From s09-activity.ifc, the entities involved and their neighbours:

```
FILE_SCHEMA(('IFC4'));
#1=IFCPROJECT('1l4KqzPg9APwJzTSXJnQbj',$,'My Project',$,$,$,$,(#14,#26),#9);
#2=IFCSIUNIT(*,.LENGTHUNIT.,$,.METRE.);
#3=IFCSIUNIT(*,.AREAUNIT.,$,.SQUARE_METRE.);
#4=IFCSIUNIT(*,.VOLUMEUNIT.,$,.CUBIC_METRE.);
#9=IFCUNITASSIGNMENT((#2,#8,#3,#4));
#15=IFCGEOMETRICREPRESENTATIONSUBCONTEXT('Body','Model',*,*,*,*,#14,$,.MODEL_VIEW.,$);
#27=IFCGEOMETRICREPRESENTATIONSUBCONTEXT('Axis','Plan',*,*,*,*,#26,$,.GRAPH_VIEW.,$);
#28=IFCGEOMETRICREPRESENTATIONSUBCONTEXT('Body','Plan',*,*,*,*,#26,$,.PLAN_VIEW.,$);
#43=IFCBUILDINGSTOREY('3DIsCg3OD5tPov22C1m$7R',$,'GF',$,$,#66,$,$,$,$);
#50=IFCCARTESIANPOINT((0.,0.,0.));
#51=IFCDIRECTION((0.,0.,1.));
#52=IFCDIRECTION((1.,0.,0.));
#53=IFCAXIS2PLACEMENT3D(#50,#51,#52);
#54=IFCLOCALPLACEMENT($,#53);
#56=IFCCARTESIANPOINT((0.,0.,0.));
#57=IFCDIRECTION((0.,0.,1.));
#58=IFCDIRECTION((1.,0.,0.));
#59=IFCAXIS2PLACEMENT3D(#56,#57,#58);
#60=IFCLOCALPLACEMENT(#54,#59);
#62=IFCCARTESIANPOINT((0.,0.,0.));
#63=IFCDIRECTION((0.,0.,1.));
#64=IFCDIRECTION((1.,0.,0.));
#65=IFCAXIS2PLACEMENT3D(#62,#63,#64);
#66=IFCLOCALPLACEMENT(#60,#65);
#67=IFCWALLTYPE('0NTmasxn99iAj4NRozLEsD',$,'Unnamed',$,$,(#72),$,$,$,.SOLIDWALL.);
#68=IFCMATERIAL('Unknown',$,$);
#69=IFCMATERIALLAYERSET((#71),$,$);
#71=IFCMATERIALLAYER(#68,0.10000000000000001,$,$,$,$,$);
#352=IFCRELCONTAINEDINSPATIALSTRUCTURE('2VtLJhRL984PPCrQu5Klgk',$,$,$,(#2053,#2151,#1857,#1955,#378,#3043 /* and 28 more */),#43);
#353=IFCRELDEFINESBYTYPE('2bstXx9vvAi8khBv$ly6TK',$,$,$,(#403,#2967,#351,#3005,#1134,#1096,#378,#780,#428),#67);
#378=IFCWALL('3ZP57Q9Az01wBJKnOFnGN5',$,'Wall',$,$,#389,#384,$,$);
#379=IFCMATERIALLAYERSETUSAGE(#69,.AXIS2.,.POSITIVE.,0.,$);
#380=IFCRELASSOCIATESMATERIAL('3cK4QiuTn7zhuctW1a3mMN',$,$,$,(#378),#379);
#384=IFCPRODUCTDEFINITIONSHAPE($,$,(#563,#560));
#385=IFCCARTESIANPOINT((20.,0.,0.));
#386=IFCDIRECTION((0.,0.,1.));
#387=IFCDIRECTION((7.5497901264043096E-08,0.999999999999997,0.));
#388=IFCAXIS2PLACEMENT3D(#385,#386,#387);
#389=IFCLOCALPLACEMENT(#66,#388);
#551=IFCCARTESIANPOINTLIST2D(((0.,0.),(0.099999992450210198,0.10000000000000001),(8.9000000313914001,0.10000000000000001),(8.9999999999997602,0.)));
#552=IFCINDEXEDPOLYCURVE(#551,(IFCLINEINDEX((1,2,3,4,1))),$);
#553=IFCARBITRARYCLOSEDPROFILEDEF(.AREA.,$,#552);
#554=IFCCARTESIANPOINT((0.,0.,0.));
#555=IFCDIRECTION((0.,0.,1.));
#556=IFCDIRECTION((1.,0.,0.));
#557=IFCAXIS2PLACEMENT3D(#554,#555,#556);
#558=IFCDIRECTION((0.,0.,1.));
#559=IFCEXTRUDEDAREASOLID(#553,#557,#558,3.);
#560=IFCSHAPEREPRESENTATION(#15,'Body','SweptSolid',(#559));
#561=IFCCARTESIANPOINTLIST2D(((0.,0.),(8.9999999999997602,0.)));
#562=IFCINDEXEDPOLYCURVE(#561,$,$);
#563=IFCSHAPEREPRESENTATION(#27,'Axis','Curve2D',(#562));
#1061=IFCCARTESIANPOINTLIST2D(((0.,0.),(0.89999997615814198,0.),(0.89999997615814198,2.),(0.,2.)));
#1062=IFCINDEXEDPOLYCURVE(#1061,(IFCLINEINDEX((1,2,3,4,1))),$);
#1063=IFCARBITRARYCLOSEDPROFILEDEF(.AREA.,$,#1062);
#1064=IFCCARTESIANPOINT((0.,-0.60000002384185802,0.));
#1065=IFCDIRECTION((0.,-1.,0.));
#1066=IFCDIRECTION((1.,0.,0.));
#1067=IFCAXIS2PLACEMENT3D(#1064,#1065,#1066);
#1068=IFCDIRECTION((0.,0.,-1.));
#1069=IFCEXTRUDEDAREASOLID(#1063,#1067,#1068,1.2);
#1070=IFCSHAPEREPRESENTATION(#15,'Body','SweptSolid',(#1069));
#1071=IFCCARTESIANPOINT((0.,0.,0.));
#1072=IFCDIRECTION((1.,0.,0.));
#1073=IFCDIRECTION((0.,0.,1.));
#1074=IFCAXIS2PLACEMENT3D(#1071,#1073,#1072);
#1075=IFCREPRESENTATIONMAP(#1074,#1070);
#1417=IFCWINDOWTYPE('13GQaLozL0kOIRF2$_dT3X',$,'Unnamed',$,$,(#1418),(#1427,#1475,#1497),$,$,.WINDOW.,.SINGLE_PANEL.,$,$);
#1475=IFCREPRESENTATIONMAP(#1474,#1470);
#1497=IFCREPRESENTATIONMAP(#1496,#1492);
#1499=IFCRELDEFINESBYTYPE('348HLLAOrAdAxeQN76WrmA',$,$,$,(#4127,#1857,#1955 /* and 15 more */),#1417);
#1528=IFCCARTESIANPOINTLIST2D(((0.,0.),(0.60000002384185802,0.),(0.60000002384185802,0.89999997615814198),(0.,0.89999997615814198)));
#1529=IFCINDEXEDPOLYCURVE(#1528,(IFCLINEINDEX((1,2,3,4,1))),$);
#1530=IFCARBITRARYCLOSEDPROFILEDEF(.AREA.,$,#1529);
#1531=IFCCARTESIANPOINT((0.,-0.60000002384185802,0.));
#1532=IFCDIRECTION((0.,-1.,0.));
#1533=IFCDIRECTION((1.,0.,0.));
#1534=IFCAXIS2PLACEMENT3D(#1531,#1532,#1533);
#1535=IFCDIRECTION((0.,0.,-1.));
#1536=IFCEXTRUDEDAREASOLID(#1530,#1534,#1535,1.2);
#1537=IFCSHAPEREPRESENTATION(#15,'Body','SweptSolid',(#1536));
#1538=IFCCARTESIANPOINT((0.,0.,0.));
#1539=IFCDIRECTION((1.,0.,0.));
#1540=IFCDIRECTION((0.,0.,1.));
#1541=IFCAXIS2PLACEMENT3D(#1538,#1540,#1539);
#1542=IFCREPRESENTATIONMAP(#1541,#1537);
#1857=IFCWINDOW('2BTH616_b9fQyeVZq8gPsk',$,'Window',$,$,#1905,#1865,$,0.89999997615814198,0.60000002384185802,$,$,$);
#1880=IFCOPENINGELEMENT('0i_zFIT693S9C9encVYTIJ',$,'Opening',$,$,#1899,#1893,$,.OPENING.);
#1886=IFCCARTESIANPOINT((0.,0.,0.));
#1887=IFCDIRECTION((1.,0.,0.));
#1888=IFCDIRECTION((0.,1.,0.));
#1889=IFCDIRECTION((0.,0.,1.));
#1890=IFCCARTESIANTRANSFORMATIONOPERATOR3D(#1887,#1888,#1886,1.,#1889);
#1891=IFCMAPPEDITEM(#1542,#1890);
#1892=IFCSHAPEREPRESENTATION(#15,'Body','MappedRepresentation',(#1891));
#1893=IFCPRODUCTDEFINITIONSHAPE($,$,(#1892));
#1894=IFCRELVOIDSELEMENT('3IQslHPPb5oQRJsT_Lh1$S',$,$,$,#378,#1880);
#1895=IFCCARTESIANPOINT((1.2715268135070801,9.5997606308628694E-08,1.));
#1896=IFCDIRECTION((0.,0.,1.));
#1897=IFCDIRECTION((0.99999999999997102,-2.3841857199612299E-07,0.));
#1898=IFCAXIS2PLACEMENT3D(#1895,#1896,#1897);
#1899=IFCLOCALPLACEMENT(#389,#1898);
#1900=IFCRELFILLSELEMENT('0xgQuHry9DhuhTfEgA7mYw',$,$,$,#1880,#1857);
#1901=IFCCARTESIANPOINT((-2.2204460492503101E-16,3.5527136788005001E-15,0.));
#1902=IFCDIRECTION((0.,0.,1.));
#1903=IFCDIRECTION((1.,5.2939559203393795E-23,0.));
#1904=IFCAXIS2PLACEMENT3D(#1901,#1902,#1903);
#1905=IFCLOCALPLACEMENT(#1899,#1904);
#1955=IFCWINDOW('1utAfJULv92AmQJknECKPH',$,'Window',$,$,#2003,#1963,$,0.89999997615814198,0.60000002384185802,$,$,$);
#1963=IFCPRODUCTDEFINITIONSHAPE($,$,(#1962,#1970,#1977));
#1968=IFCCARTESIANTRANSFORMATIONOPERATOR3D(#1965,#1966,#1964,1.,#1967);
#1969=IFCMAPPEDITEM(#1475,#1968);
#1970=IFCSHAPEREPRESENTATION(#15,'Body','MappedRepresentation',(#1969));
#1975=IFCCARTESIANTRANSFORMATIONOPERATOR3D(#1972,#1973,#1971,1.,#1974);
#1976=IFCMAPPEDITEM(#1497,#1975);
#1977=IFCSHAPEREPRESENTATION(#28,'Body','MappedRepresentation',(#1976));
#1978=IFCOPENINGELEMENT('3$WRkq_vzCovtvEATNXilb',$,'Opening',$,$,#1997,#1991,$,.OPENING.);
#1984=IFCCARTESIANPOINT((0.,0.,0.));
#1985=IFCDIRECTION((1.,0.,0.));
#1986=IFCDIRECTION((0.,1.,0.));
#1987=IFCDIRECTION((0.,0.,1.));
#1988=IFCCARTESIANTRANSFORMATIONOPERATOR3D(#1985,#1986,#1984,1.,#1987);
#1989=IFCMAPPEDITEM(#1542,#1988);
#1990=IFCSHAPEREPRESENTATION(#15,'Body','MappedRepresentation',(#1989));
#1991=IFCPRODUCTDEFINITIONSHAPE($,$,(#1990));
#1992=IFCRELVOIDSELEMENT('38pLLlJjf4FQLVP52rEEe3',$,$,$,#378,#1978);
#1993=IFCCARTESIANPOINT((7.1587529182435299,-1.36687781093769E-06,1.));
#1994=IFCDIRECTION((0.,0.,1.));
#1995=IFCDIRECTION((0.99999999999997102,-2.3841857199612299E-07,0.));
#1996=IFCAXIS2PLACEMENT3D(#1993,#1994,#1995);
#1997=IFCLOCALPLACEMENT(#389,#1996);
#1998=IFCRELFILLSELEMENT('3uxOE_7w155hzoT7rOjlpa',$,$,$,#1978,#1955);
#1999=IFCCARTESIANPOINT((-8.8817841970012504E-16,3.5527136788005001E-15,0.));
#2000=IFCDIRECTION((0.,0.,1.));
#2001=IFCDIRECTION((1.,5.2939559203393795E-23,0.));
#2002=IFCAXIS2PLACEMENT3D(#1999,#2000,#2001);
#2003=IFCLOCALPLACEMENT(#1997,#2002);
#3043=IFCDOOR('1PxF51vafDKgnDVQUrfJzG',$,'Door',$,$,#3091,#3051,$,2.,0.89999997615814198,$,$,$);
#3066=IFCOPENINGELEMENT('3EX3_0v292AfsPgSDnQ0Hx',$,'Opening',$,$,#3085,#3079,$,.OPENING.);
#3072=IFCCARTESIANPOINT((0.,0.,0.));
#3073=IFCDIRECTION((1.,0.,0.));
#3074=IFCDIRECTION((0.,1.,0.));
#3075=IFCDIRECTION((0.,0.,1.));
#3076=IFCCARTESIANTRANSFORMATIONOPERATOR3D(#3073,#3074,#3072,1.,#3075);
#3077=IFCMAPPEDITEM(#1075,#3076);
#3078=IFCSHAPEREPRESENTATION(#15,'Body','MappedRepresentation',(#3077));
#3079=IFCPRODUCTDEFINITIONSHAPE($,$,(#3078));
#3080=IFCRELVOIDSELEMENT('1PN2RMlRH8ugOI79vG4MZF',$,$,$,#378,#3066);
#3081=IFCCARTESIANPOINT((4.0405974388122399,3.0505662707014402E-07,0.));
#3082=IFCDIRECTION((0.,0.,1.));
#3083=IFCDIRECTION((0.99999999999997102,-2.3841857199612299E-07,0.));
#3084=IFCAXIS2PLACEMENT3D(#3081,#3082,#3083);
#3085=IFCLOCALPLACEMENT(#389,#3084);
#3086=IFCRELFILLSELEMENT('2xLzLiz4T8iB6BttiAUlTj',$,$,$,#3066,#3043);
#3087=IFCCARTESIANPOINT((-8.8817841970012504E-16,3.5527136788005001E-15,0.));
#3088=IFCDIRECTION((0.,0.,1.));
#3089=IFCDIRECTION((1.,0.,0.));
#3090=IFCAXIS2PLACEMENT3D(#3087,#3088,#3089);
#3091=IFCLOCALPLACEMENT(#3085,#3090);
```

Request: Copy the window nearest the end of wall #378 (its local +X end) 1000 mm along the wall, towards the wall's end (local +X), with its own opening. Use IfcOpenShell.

```python
import ifcopenshell
import ifcopenshell.api.feature
import ifcopenshell.api.geometry
import ifcopenshell.api.root
import ifcopenshell.geom
import ifcopenshell.util.element
import ifcopenshell.util.placement
import ifcopenshell.util.shape
import ifcopenshell.util.unit

model = ifcopenshell.open("s09-activity.ifc")
unit_scale = ifcopenshell.util.unit.calculate_unit_scale(model)
settings = ifcopenshell.geom.settings()


def volume(element):
    """Net volume in cubic metres, openings subtracted."""
    shape = ifcopenshell.geom.create_shape(settings, element)
    return ifcopenshell.util.shape.get_volume(shape.geometry)


window = model.by_id(1955)
opening = window.FillsVoids[0].RelatingOpeningElement
wall = opening.VoidsElements[0].RelatingBuildingElement
before = volume(wall)
shift = ifcopenshell.util.placement.get_local_placement(wall.ObjectPlacement)[:3, 0] * 1 / unit_scale

# copy_class copies the void relationship, type, container and properties, but no geometry.
new_opening = ifcopenshell.api.root.copy_class(model, product=opening)
new_opening.Representation = ifcopenshell.util.element.copy_deep(
    model, opening.Representation, exclude=["IfcGeometricRepresentationContext", "IfcRepresentationMap"]
)
new_window = ifcopenshell.api.root.copy_class(model, product=window)
new_window.Representation = ifcopenshell.util.element.copy_deep(
    model, window.Representation, exclude=["IfcGeometricRepresentationContext", "IfcRepresentationMap"]
)
ifcopenshell.api.feature.add_filling(model, opening=new_opening, element=new_window)

for old, new in ((opening, new_opening), (window, new_window)):
    matrix = ifcopenshell.util.placement.get_local_placement(old.ObjectPlacement)
    matrix[:3, 3] += shift
    ifcopenshell.api.geometry.edit_object_placement(model, product=new, matrix=matrix, is_si=False)

after = volume(wall)

print(f"wall volume {before:.3f} -> {after:.3f} m3")

model.write("s09-activity-out.ifc")
```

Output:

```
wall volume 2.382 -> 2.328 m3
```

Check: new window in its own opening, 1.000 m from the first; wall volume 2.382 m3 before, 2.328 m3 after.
